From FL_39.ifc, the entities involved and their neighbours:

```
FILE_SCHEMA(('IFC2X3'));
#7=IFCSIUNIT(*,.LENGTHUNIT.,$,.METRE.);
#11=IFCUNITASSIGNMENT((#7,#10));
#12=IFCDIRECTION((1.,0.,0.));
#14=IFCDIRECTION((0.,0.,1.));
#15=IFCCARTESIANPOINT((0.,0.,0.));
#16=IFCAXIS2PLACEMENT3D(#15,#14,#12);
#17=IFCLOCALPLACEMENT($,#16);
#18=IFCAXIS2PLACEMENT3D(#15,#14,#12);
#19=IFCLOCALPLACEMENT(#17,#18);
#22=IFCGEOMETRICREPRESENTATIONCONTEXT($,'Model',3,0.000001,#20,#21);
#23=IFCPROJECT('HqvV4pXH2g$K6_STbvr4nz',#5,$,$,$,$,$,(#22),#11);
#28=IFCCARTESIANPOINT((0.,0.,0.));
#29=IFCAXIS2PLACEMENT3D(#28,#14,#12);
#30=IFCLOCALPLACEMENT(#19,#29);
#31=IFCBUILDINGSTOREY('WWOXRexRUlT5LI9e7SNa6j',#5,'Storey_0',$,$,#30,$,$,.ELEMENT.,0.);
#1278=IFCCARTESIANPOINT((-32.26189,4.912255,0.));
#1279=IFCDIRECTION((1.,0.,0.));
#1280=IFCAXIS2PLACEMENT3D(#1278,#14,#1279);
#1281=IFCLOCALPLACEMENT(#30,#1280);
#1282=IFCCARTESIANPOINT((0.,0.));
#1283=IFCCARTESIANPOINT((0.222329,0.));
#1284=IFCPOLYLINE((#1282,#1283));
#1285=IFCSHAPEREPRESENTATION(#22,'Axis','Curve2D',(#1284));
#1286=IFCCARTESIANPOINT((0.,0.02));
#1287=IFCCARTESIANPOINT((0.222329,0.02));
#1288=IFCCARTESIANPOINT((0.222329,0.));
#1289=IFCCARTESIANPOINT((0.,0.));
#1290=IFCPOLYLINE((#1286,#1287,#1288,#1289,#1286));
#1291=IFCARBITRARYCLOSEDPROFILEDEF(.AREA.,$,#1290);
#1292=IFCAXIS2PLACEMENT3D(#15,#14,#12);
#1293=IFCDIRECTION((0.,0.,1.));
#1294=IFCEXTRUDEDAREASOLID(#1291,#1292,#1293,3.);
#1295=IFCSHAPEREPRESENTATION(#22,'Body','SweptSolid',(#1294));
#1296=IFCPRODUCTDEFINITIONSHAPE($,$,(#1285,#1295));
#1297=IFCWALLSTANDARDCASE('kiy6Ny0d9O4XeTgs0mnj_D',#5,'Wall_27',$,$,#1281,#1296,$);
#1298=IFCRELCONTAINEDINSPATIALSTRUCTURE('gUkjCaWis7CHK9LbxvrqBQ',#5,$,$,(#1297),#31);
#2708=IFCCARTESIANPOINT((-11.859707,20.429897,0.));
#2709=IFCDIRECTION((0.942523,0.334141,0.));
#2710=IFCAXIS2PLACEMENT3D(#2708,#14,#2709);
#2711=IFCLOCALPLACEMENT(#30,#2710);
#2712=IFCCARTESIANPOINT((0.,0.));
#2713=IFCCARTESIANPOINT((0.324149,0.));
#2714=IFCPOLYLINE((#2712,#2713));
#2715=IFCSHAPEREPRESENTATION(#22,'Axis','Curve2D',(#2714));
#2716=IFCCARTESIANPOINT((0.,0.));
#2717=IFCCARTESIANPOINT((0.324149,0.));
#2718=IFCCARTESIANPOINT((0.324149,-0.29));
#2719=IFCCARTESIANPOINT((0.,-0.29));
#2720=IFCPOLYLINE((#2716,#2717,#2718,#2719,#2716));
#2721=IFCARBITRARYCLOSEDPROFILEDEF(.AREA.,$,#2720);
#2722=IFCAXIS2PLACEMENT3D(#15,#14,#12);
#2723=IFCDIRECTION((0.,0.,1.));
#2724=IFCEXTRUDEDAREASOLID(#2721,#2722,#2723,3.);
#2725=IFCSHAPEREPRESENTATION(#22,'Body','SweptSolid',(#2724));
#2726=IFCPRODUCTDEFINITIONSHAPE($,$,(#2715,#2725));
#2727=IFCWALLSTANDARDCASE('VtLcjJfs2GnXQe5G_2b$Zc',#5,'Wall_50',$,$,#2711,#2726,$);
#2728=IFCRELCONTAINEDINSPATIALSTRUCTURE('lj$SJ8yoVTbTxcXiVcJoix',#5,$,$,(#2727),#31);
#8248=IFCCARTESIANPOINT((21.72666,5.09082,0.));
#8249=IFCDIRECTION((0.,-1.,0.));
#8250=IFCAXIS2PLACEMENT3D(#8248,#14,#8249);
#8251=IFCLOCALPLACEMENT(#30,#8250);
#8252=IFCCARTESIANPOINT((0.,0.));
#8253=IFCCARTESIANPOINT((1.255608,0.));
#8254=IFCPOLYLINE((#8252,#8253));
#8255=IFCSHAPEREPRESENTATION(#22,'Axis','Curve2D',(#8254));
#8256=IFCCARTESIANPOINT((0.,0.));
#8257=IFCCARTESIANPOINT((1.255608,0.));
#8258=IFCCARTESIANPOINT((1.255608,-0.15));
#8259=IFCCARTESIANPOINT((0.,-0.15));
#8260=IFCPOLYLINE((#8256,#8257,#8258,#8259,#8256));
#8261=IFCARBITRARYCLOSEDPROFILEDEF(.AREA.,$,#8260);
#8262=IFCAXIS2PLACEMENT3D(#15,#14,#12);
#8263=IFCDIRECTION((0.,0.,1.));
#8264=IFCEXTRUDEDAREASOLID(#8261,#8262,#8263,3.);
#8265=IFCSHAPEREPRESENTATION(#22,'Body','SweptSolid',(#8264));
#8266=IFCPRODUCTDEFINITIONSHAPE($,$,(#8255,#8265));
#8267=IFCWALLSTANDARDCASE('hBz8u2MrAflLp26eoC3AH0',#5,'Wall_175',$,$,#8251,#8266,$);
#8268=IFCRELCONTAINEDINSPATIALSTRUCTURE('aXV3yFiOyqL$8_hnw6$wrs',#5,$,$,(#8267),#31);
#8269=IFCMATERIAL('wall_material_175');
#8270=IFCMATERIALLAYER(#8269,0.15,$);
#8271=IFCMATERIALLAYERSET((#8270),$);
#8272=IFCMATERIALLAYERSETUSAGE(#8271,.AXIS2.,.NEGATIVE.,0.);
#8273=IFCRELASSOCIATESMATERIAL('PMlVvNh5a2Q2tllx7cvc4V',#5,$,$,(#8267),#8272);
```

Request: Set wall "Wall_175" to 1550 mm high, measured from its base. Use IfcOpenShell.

```python
import ifcopenshell
import ifcopenshell.geom
import ifcopenshell.util.shape
import ifcopenshell.util.unit

model = ifcopenshell.open("FL_39.ifc")
unit_scale = ifcopenshell.util.unit.calculate_unit_scale(model)
settings = ifcopenshell.geom.settings()


def volume(element):
    """Net volume in cubic metres, openings subtracted."""
    shape = ifcopenshell.geom.create_shape(settings, element)
    return ifcopenshell.util.shape.get_volume(shape.geometry)


wall = model.by_id(8267)
before = volume(wall)

body = next(r for r in wall.Representation.Representations if r.RepresentationIdentifier == "Body")
solid = body.Items[0]
old_height = solid.Depth
solid.Depth = 1.55 / unit_scale
after = volume(wall)

print(f"height {old_height:g} -> {solid.Depth:g}, volume {before:.3f} -> {after:.3f} m3")

model.write("FL_39_rev.ifc")
```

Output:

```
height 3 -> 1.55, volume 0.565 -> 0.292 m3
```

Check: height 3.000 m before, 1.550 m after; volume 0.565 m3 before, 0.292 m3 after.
